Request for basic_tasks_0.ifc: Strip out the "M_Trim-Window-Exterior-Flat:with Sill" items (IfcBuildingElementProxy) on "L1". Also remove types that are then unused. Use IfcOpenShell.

First a look at what the model holds.

```python
import ifcopenshell
import ifcopenshell.util.element

model = ifcopenshell.open("basic_tasks_0.ifc")
print(model.schema)
storey = next(s for s in model.by_type("IfcBuildingStorey") if s.Name == "L1")
proxies = [e for e in ifcopenshell.util.element.get_decomposition(storey) if e.is_a("IfcBuildingElementProxy")]
seen = {}
for e in proxies:
    element_type = ifcopenshell.util.element.get_type(e)
    name = element_type.Name if element_type not in (None, e) else None
    seen[name] = seen.get(name, 0) + 1
for name, count in sorted(seen.items(), key=str):
    print(count, "x", name)
```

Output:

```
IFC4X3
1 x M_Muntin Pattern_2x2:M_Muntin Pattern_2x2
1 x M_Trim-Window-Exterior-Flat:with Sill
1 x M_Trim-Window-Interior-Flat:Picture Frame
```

```python
import ifcopenshell
import ifcopenshell.api.root
import ifcopenshell.util.element

model = ifcopenshell.open("basic_tasks_0.ifc")

storey = next(s for s in model.by_type("IfcBuildingStorey") if s.Name == "L1")
proxies = [e for e in ifcopenshell.util.element.get_decomposition(storey) if e.is_a("IfcBuildingElementProxy")]
targets = [e for e in proxies if (t := ifcopenshell.util.element.get_type(e)) not in (None, e) and t.Name == "M_Trim-Window-Exterior-Flat:with Sill"]
types = {ifcopenshell.util.element.get_type(e) for e in targets} - {None, *targets}

for e in targets:
    ifcopenshell.api.root.remove_product(model, product=e)
print(len(targets), "removed")

unused = [t for t in types if not ifcopenshell.util.element.get_types(t)]
for t in unused:
    ifcopenshell.api.root.remove_product(model, product=t)
print(len(unused), "unused types removed")

model.write("basic_tasks_0_v2.ifc")
```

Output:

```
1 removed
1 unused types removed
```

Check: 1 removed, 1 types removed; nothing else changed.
